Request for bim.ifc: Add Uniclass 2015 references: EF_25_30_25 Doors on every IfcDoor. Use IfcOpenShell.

First a look at what the model holds.

```python
import ifcopenshell

model = ifcopenshell.open("bim.ifc")
print(model.schema)
print("classifications:", [c.Name for c in model.by_type("IfcClassification")])
for ifc_class in ("IfcDoor", "IfcRoof", "IfcStair", "IfcWall", "IfcWindow"):
    print(ifc_class, len(model.by_type(ifc_class)))
```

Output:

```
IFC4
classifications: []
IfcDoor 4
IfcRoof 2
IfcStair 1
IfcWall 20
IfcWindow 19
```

```python
import ifcopenshell
import ifcopenshell.api.classification

model = ifcopenshell.open("bim.ifc")

system = ifcopenshell.api.classification.add_classification(model, classification="Uniclass 2015")

codes = {
    "IfcDoor": ("EF_25_30_25", "Doors"),
}
for ifc_class, (code, name) in codes.items():
    products = model.by_type(ifc_class)
    ifcopenshell.api.classification.add_reference(
        model, products=products, classification=system, identification=code, name=name
    )
    print(code, len(products))

model.write("bim_edited.ifc")
```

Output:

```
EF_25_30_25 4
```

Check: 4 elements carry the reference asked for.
